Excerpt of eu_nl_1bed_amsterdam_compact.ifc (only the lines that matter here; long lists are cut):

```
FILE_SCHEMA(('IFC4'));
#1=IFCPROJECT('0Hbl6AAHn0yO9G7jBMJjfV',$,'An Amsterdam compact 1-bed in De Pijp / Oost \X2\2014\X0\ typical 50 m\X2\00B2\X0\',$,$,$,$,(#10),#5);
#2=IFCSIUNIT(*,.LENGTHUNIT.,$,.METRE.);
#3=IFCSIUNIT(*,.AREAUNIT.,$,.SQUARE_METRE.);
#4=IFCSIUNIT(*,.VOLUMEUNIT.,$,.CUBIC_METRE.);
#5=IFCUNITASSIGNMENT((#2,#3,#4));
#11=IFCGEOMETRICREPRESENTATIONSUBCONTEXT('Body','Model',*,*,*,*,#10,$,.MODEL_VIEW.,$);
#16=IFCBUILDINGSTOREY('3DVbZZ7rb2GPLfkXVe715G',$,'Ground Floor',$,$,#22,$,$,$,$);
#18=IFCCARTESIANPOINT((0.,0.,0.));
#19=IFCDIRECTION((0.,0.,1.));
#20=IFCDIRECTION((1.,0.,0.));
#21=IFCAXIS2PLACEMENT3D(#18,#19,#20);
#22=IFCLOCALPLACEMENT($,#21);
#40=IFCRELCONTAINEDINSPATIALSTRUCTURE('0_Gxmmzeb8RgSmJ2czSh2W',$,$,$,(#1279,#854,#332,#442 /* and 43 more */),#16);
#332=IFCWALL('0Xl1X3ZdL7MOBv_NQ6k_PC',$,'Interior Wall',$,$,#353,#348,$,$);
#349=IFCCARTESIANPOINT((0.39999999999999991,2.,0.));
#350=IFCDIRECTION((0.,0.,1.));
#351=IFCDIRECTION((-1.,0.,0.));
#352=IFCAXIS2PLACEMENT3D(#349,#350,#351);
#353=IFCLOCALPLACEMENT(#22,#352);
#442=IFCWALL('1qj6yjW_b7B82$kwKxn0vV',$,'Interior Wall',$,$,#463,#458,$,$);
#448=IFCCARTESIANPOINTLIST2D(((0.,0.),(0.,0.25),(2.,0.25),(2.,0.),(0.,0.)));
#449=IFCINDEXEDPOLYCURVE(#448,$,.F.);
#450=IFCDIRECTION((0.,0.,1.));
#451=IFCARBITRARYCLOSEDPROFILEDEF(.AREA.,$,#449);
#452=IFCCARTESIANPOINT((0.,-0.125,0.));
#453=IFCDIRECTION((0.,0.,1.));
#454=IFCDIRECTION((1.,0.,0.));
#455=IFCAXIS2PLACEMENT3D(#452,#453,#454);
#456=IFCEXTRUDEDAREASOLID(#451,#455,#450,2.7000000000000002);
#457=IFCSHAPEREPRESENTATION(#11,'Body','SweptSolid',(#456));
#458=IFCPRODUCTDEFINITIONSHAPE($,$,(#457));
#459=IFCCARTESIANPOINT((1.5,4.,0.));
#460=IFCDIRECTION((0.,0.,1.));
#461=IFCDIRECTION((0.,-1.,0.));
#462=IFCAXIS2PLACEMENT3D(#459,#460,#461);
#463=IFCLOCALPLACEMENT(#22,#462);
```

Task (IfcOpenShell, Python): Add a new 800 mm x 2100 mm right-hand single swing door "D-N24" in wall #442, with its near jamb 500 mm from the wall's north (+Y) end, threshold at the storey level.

```python
import numpy as np
import ifcopenshell
import ifcopenshell.api.feature
import ifcopenshell.api.geometry
import ifcopenshell.api.root
import ifcopenshell.api.spatial
import ifcopenshell.geom
import ifcopenshell.util.element
import ifcopenshell.util.placement
import ifcopenshell.util.representation
import ifcopenshell.util.shape
import ifcopenshell.util.unit

model = ifcopenshell.open("eu_nl_1bed_amsterdam_compact.ifc")
unit_scale = ifcopenshell.util.unit.calculate_unit_scale(model)
settings = ifcopenshell.geom.settings()


def volume(element):
    """Net volume in cubic metres, openings subtracted."""
    shape = ifcopenshell.geom.create_shape(settings, element)
    return ifcopenshell.util.shape.get_volume(shape.geometry)


wall = model.by_guid("1qj6yjW_b7B82$kwKxn0vV")
storey = ifcopenshell.util.element.get_container(wall, ifc_class="IfcBuildingStorey")
context = ifcopenshell.util.representation.get_context(model, "Model", "Body", "MODEL_VIEW")
before = volume(wall)

width, height, from_end, sill = 0.8, 2.1, 0.5, 0.0  # metres

# The wall runs along its own X axis, and the end named is its -X end.
wall_shape = ifcopenshell.geom.create_shape(settings, wall)
x, y, z = ifcopenshell.util.shape.get_vertices(wall_shape.geometry).T
start = x.min() + from_end
face, thickness = float(y.min()), float(y.max() - y.min())
wall_matrix = ifcopenshell.util.placement.get_local_placement(wall.ObjectPlacement)
level = ifcopenshell.util.placement.get_local_placement(storey.ObjectPlacement)[2, 3]


def in_wall(x, y):
    """Placement at x, y metres in the wall's axes, at sill height."""
    matrix = wall_matrix.copy()
    matrix[:, 3] = wall_matrix @ np.array([x / unit_scale, y / unit_scale, 0.0, 1.0])
    matrix[2, 3] = level + sill / unit_scale
    return matrix


# Opening: a box that overshoots both wall faces by 50 mm.
opening = ifcopenshell.api.root.create_entity(model, ifc_class="IfcOpeningElement", predefined_type="OPENING")
box = ifcopenshell.api.geometry.add_wall_representation(
    model, context=context, length=width, height=height, thickness=thickness + 0.1
)
ifcopenshell.api.geometry.assign_representation(model, product=opening, representation=box)
ifcopenshell.api.geometry.edit_object_placement(model, product=opening, matrix=in_wall(start, face - 0.05), is_si=False)
ifcopenshell.api.feature.add_feature(model, feature=opening, element=wall)

door = ifcopenshell.api.root.create_entity(model, ifc_class="IfcDoor", name="D-N24", predefined_type="DOOR")
door.OverallWidth, door.OverallHeight = width / unit_scale, height / unit_scale
door.OperationType = "SINGLE_SWING_RIGHT"
body = ifcopenshell.api.geometry.add_door_representation(
    model,
    context=context,
    overall_width=door.OverallWidth,
    overall_height=door.OverallHeight,
    operation_type="SINGLE_SWING_RIGHT",
    lining_properties={"LiningDepth": thickness / unit_scale, "ThresholdDepth": thickness / unit_scale},
)
ifcopenshell.api.geometry.assign_representation(model, product=door, representation=body)
ifcopenshell.api.spatial.assign_container(model, products=[door], relating_structure=storey)
ifcopenshell.api.feature.add_filling(model, opening=opening, element=door)

# The lining spans the wall, so the door starts at the wall face.
ifcopenshell.api.geometry.edit_object_placement(model, product=door, matrix=in_wall(start, face), is_si=False)

after = volume(wall)

print(f"wall volume {before:.3f} -> {after:.3f} m3")

model.write("eu_nl_1bed_amsterdam_compact_v2.ifc")
```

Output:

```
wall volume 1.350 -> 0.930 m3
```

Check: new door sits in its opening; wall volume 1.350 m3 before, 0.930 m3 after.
